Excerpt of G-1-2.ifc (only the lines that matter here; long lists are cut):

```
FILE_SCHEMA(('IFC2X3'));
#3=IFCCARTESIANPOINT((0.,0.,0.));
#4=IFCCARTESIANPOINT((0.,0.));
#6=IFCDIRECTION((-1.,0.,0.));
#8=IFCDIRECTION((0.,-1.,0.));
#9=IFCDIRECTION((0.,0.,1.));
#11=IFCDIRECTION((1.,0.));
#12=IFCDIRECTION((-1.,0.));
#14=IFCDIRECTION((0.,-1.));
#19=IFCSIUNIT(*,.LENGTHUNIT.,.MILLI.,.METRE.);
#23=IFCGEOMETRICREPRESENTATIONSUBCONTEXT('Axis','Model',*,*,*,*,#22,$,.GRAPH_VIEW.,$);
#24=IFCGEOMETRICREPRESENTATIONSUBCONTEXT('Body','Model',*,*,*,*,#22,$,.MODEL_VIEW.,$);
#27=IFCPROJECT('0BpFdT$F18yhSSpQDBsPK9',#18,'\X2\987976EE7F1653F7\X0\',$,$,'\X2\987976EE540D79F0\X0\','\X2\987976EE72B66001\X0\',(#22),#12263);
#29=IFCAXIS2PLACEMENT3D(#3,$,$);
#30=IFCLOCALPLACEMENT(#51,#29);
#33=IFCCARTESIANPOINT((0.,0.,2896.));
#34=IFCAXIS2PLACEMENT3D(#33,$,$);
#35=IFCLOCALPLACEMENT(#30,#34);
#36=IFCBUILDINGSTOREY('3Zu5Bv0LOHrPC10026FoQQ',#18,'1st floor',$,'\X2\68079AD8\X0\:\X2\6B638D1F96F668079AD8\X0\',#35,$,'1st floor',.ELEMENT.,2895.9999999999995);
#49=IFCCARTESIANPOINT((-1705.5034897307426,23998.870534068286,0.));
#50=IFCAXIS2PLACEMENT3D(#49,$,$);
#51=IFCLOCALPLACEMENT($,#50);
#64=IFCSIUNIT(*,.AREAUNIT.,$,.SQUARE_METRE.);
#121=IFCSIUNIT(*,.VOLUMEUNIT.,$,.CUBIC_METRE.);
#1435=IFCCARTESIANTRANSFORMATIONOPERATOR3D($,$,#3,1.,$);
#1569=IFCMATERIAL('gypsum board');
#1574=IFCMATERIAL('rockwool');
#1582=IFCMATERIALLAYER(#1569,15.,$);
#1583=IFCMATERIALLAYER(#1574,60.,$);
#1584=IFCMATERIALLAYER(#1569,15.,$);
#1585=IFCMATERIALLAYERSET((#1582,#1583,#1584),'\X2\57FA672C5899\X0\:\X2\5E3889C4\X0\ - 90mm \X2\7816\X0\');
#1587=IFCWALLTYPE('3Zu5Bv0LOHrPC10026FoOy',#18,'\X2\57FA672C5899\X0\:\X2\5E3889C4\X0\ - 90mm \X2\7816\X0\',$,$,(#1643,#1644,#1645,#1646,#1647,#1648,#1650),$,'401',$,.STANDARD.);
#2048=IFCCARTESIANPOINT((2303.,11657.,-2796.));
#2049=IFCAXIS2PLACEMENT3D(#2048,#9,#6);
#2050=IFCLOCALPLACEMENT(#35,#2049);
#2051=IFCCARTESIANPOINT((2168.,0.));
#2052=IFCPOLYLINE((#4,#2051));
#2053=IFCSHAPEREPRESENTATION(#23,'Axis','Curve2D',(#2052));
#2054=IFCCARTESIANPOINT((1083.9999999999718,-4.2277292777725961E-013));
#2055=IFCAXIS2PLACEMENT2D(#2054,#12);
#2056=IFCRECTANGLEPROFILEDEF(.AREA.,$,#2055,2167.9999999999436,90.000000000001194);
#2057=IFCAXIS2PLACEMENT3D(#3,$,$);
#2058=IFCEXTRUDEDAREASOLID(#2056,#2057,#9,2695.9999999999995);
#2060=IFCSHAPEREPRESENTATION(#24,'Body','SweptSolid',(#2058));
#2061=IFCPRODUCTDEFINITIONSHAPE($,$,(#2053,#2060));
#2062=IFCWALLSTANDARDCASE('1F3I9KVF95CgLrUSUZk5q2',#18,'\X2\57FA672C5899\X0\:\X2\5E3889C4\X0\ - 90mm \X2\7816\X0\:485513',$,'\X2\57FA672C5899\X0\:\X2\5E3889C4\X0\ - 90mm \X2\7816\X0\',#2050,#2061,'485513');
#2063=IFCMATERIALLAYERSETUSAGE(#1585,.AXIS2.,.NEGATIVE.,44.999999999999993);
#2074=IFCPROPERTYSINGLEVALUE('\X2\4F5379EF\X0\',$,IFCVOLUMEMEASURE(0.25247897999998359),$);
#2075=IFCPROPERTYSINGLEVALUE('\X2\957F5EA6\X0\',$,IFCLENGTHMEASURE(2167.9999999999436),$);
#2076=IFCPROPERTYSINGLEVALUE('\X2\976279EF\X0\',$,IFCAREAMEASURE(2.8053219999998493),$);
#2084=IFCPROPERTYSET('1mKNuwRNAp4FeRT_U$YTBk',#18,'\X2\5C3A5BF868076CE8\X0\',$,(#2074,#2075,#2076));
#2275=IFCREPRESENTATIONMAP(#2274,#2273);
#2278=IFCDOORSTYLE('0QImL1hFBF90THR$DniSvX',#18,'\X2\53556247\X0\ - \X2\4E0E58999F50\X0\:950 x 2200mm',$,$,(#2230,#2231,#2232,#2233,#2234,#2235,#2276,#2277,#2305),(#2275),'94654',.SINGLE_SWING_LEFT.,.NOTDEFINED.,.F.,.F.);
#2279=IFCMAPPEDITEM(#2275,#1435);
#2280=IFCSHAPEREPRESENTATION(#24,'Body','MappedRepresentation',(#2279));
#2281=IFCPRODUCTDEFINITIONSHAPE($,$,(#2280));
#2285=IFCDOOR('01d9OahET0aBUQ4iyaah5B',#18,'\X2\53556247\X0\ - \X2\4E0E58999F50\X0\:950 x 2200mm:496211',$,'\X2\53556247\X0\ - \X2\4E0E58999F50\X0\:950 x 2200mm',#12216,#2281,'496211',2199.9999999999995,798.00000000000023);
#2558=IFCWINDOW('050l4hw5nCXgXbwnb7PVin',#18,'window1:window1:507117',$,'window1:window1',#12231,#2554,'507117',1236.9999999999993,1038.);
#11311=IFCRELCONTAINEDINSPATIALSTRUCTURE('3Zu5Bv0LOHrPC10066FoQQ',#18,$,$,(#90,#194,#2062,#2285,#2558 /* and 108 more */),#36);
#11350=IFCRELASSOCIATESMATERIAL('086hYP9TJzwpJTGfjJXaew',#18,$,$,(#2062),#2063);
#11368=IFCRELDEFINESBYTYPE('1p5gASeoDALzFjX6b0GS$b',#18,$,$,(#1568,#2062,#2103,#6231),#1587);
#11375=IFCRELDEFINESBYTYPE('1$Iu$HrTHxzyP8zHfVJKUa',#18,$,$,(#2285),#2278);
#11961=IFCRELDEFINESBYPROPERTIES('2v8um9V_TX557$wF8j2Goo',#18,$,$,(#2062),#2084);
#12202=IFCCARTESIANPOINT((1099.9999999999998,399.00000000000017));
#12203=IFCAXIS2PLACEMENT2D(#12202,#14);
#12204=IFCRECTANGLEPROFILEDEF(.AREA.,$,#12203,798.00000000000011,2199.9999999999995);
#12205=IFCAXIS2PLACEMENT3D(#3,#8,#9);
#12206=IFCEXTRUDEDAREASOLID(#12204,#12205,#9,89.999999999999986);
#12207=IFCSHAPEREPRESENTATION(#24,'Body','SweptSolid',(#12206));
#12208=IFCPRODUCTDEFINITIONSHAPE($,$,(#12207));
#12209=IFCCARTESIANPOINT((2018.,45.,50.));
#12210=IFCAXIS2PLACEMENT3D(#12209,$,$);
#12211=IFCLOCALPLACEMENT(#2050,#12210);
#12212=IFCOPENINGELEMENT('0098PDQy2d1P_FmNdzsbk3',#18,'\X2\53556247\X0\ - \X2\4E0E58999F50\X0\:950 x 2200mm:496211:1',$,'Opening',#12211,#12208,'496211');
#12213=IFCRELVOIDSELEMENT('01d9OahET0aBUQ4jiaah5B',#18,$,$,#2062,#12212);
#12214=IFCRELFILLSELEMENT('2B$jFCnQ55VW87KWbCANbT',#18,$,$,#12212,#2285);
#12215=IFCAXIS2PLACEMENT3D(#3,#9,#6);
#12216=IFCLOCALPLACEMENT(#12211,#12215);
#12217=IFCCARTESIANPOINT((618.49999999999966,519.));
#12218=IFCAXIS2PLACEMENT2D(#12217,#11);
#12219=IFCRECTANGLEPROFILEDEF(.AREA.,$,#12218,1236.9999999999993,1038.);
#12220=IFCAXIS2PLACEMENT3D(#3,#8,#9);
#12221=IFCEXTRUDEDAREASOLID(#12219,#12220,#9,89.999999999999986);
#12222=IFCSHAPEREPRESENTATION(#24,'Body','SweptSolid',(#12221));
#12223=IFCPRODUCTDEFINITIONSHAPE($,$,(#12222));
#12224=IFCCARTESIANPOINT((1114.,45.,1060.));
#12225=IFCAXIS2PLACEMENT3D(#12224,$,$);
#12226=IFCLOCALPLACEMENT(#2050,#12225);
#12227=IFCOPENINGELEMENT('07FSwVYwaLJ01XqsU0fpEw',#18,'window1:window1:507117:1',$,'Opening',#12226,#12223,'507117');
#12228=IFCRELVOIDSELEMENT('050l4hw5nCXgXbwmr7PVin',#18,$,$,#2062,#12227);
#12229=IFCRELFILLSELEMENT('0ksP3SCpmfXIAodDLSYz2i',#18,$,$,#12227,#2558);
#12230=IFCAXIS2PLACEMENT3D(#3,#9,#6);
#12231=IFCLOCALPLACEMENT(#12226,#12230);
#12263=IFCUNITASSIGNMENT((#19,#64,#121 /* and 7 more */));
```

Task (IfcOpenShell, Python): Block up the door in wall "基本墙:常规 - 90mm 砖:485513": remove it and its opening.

```python
import ifcopenshell
import ifcopenshell.api.feature
import ifcopenshell.api.pset
import ifcopenshell.api.root
import ifcopenshell.geom
import ifcopenshell.util.element
import ifcopenshell.util.shape
import ifcopenshell.util.unit

model = ifcopenshell.open("G-1-2.ifc")
area_scale = ifcopenshell.util.unit.calculate_unit_scale(model, "AREAUNIT")
volume_scale = ifcopenshell.util.unit.calculate_unit_scale(model, "VOLUMEUNIT")
settings = ifcopenshell.geom.settings()


def volume(element):
    """Net volume in cubic metres, openings subtracted."""
    shape = ifcopenshell.geom.create_shape(settings, element)
    return ifcopenshell.util.shape.get_volume(shape.geometry)


door = model.by_guid("01d9OahET0aBUQ4iyaah5B")
opening = door.FillsVoids[0].RelatingOpeningElement
wall = opening.VoidsElements[0].RelatingBuildingElement
before = volume(wall)

ifcopenshell.api.root.remove_product(model, product=door)
ifcopenshell.api.feature.remove_feature(model, feature=opening)

after = volume(wall)
thickness = 0.09  # wall thickness in metres

# Update the wall's stored quantities.
pset = model.by_id(ifcopenshell.util.element.get_pset(wall, "尺寸标注", should_inherit=False)["id"])
ifcopenshell.api.pset.edit_pset(model, pset=pset, properties={
    "体积": model.create_entity("IfcVolumeMeasure", after / volume_scale),
    "面积": model.create_entity("IfcAreaMeasure", after / thickness / area_scale),
})

print(f"wall volume {before:.3f} -> {after:.3f} m3")

model.write("G-1-2_rev.ifc")
```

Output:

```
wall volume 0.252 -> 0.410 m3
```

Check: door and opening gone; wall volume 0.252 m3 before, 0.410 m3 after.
